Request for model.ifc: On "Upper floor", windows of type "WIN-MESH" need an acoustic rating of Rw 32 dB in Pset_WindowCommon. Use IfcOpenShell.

First a look at what the model holds.

```python
import ifcopenshell
import ifcopenshell.util.element

model = ifcopenshell.open("model.ifc")
print(model.schema)
storey = next(s for s in model.by_type("IfcBuildingStorey") if s.Name == "Upper floor")
windows = [e for e in ifcopenshell.util.element.get_decomposition(storey) if e.is_a("IfcWindow")]
seen = {}
for e in windows:
    element_type = ifcopenshell.util.element.get_type(e)
    key = (element_type.Name if element_type != e and element_type else None, ifcopenshell.util.element.get_pset(e, "Pset_WindowCommon", "AcousticRating"))
    seen[key] = seen.get(key, 0) + 1
for (name, value), count in sorted(seen.items(), key=str):
    print(count, "x", name, "|", value)
```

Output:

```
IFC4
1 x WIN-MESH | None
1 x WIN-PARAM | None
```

```python
import ifcopenshell
import ifcopenshell.api.pset
import ifcopenshell.util.element

model = ifcopenshell.open("model.ifc")

storey = next(s for s in model.by_type("IfcBuildingStorey") if s.Name == "Upper floor")
windows = [e for e in ifcopenshell.util.element.get_decomposition(storey) if e.is_a("IfcWindow")]

count = 0
for e in windows:
    element_type = ifcopenshell.util.element.get_type(e)
    if element_type in (None, e) or element_type.Name != "WIN-MESH":
        continue
    # add_pset returns the element's existing set when there is one.
    pset = ifcopenshell.api.pset.add_pset(model, product=e, name="Pset_WindowCommon")
    ifcopenshell.api.pset.edit_pset(model, pset=pset, properties={"AcousticRating": "Rw 32 dB"})
    count += 1

print(count, "windows updated")

model.write("model_rev.ifc")
```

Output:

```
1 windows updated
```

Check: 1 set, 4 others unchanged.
